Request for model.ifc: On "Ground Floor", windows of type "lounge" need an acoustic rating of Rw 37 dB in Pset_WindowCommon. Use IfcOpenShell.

First a look at what the model holds.

```python
import ifcopenshell
import ifcopenshell.util.element

model = ifcopenshell.open("model.ifc")
print(model.schema)
storey = next(s for s in model.by_type("IfcBuildingStorey") if s.Name == "Ground Floor")
windows = [e for e in ifcopenshell.util.element.get_decomposition(storey) if e.is_a("IfcWindow")]
seen = {}
for e in windows:
    element_type = ifcopenshell.util.element.get_type(e)
    key = (element_type.Name if element_type != e and element_type else None, ifcopenshell.util.element.get_pset(e, "Pset_WindowCommon", "AcousticRating"))
    seen[key] = seen.get(key, 0) + 1
for (name, value), count in sorted(seen.items(), key=str):
    print(count, "x", name, "|", value)
```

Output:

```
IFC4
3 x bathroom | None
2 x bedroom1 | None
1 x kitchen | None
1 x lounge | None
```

```python
import ifcopenshell
import ifcopenshell.api.pset
import ifcopenshell.util.element

model = ifcopenshell.open("model.ifc")

storey = next(s for s in model.by_type("IfcBuildingStorey") if s.Name == "Ground Floor")
windows = [e for e in ifcopenshell.util.element.get_decomposition(storey) if e.is_a("IfcWindow")]

count = 0
for e in windows:
    element_type = ifcopenshell.util.element.get_type(e)
    if element_type in (None, e) or element_type.Name != "lounge":
        continue
    # add_pset returns the element's existing set when there is one.
    pset = ifcopenshell.api.pset.add_pset(model, product=e, name="Pset_WindowCommon")
    ifcopenshell.api.pset.edit_pset(model, pset=pset, properties={"AcousticRating": "Rw 37 dB"})
    count += 1

print(count, "windows updated")

model.write("model_updated.ifc")
```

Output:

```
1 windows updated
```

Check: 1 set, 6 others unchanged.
